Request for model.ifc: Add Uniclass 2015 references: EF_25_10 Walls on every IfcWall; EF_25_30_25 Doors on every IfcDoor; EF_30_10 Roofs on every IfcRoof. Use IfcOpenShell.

First a look at what the model holds.

```python
import ifcopenshell

model = ifcopenshell.open("model.ifc")
print(model.schema)
print("classifications:", [c.Name for c in model.by_type("IfcClassification")])
for ifc_class in ("IfcDoor", "IfcRoof", "IfcStair", "IfcWall", "IfcWindow"):
    print(ifc_class, len(model.by_type(ifc_class)))
```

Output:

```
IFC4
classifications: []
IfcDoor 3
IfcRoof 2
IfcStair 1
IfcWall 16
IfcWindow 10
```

```python
import ifcopenshell
import ifcopenshell.api.classification

model = ifcopenshell.open("model.ifc")

system = ifcopenshell.api.classification.add_classification(model, classification="Uniclass 2015")

codes = {
    "IfcWall": ("EF_25_10", "Walls"),
    "IfcDoor": ("EF_25_30_25", "Doors"),
    "IfcRoof": ("EF_30_10", "Roofs"),
}
for ifc_class, (code, name) in codes.items():
    products = model.by_type(ifc_class)
    ifcopenshell.api.classification.add_reference(
        model, products=products, classification=system, identification=code, name=name
    )
    print(code, len(products))

model.write("model-out.ifc")
```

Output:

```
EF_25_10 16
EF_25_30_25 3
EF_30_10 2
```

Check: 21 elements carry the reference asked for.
